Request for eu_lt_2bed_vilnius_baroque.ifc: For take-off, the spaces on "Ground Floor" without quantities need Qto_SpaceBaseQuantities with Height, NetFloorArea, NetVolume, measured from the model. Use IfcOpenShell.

First a look at what the model holds.

```python
import ifcopenshell
import ifcopenshell.util.element
import ifcopenshell.util.unit

model = ifcopenshell.open("eu_lt_2bed_vilnius_baroque.ifc")
print(model.schema)
for unit_type in ("LENGTHUNIT", "AREAUNIT", "VOLUMEUNIT"):
    print(unit_type, ifcopenshell.util.unit.calculate_unit_scale(model, unit_type))
storey = next(s for s in model.by_type("IfcBuildingStorey") if s.Name == "Ground Floor")
spaces = [e for e in ifcopenshell.util.element.get_decomposition(storey) if e.is_a("IfcSpace")]
for e in sorted(spaces, key=lambda e: e.id()):
    print(e.id(), e.is_a(), e.Name, list(ifcopenshell.util.element.get_psets(e, qtos_only=True)), sep=" | ")
```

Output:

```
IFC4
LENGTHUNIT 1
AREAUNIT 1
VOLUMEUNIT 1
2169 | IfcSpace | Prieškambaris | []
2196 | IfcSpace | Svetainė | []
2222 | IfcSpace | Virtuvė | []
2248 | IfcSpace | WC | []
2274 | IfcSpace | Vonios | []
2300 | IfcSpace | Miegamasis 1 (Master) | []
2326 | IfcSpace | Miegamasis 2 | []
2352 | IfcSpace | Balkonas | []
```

```python
import ifcopenshell
import ifcopenshell.api.pset
import ifcopenshell.geom
import ifcopenshell.util.element
import ifcopenshell.util.shape
import ifcopenshell.util.unit

model = ifcopenshell.open("eu_lt_2bed_vilnius_baroque.ifc")
unit_scale = ifcopenshell.util.unit.calculate_unit_scale(model)
area_scale = ifcopenshell.util.unit.calculate_unit_scale(model, "AREAUNIT")
volume_scale = ifcopenshell.util.unit.calculate_unit_scale(model, "VOLUMEUNIT")
settings = ifcopenshell.geom.settings()

storey = next(s for s in model.by_type("IfcBuildingStorey") if s.Name == "Ground Floor")
spaces = [e for e in ifcopenshell.util.element.get_decomposition(storey) if e.is_a("IfcSpace")]

for e in sorted(spaces, key=lambda e: e.id()):
    if ifcopenshell.util.element.get_psets(e, qtos_only=True, should_inherit=False):
        continue
    # Geometry comes back in metres, in the element's own axes.
    shape = ifcopenshell.geom.create_shape(settings, e)
    values = {
        "Height": ifcopenshell.util.shape.get_z(shape.geometry) / unit_scale,
        "NetFloorArea": ifcopenshell.util.shape.get_footprint_area(shape.geometry) / area_scale,
        "NetVolume": ifcopenshell.util.shape.get_volume(shape.geometry) / volume_scale,
    }
    qto = ifcopenshell.api.pset.add_qto(model, product=e, name="Qto_SpaceBaseQuantities")
    ifcopenshell.api.pset.edit_qto(model, qto=qto, properties=values)
    print(e.id(), {k: round(v, 3) for k, v in values.items()})

model.write("eu_lt_2bed_vilnius_baroque_edited.ifc")
```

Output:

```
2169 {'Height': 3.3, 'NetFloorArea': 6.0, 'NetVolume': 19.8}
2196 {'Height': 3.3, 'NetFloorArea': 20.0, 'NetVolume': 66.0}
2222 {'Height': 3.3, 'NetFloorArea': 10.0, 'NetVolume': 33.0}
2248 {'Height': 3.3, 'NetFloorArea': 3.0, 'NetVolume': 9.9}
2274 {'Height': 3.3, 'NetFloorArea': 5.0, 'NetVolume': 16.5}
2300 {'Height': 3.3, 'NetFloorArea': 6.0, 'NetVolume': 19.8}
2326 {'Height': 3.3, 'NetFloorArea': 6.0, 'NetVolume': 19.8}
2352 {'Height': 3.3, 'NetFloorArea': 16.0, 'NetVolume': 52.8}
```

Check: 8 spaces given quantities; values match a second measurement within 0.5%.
